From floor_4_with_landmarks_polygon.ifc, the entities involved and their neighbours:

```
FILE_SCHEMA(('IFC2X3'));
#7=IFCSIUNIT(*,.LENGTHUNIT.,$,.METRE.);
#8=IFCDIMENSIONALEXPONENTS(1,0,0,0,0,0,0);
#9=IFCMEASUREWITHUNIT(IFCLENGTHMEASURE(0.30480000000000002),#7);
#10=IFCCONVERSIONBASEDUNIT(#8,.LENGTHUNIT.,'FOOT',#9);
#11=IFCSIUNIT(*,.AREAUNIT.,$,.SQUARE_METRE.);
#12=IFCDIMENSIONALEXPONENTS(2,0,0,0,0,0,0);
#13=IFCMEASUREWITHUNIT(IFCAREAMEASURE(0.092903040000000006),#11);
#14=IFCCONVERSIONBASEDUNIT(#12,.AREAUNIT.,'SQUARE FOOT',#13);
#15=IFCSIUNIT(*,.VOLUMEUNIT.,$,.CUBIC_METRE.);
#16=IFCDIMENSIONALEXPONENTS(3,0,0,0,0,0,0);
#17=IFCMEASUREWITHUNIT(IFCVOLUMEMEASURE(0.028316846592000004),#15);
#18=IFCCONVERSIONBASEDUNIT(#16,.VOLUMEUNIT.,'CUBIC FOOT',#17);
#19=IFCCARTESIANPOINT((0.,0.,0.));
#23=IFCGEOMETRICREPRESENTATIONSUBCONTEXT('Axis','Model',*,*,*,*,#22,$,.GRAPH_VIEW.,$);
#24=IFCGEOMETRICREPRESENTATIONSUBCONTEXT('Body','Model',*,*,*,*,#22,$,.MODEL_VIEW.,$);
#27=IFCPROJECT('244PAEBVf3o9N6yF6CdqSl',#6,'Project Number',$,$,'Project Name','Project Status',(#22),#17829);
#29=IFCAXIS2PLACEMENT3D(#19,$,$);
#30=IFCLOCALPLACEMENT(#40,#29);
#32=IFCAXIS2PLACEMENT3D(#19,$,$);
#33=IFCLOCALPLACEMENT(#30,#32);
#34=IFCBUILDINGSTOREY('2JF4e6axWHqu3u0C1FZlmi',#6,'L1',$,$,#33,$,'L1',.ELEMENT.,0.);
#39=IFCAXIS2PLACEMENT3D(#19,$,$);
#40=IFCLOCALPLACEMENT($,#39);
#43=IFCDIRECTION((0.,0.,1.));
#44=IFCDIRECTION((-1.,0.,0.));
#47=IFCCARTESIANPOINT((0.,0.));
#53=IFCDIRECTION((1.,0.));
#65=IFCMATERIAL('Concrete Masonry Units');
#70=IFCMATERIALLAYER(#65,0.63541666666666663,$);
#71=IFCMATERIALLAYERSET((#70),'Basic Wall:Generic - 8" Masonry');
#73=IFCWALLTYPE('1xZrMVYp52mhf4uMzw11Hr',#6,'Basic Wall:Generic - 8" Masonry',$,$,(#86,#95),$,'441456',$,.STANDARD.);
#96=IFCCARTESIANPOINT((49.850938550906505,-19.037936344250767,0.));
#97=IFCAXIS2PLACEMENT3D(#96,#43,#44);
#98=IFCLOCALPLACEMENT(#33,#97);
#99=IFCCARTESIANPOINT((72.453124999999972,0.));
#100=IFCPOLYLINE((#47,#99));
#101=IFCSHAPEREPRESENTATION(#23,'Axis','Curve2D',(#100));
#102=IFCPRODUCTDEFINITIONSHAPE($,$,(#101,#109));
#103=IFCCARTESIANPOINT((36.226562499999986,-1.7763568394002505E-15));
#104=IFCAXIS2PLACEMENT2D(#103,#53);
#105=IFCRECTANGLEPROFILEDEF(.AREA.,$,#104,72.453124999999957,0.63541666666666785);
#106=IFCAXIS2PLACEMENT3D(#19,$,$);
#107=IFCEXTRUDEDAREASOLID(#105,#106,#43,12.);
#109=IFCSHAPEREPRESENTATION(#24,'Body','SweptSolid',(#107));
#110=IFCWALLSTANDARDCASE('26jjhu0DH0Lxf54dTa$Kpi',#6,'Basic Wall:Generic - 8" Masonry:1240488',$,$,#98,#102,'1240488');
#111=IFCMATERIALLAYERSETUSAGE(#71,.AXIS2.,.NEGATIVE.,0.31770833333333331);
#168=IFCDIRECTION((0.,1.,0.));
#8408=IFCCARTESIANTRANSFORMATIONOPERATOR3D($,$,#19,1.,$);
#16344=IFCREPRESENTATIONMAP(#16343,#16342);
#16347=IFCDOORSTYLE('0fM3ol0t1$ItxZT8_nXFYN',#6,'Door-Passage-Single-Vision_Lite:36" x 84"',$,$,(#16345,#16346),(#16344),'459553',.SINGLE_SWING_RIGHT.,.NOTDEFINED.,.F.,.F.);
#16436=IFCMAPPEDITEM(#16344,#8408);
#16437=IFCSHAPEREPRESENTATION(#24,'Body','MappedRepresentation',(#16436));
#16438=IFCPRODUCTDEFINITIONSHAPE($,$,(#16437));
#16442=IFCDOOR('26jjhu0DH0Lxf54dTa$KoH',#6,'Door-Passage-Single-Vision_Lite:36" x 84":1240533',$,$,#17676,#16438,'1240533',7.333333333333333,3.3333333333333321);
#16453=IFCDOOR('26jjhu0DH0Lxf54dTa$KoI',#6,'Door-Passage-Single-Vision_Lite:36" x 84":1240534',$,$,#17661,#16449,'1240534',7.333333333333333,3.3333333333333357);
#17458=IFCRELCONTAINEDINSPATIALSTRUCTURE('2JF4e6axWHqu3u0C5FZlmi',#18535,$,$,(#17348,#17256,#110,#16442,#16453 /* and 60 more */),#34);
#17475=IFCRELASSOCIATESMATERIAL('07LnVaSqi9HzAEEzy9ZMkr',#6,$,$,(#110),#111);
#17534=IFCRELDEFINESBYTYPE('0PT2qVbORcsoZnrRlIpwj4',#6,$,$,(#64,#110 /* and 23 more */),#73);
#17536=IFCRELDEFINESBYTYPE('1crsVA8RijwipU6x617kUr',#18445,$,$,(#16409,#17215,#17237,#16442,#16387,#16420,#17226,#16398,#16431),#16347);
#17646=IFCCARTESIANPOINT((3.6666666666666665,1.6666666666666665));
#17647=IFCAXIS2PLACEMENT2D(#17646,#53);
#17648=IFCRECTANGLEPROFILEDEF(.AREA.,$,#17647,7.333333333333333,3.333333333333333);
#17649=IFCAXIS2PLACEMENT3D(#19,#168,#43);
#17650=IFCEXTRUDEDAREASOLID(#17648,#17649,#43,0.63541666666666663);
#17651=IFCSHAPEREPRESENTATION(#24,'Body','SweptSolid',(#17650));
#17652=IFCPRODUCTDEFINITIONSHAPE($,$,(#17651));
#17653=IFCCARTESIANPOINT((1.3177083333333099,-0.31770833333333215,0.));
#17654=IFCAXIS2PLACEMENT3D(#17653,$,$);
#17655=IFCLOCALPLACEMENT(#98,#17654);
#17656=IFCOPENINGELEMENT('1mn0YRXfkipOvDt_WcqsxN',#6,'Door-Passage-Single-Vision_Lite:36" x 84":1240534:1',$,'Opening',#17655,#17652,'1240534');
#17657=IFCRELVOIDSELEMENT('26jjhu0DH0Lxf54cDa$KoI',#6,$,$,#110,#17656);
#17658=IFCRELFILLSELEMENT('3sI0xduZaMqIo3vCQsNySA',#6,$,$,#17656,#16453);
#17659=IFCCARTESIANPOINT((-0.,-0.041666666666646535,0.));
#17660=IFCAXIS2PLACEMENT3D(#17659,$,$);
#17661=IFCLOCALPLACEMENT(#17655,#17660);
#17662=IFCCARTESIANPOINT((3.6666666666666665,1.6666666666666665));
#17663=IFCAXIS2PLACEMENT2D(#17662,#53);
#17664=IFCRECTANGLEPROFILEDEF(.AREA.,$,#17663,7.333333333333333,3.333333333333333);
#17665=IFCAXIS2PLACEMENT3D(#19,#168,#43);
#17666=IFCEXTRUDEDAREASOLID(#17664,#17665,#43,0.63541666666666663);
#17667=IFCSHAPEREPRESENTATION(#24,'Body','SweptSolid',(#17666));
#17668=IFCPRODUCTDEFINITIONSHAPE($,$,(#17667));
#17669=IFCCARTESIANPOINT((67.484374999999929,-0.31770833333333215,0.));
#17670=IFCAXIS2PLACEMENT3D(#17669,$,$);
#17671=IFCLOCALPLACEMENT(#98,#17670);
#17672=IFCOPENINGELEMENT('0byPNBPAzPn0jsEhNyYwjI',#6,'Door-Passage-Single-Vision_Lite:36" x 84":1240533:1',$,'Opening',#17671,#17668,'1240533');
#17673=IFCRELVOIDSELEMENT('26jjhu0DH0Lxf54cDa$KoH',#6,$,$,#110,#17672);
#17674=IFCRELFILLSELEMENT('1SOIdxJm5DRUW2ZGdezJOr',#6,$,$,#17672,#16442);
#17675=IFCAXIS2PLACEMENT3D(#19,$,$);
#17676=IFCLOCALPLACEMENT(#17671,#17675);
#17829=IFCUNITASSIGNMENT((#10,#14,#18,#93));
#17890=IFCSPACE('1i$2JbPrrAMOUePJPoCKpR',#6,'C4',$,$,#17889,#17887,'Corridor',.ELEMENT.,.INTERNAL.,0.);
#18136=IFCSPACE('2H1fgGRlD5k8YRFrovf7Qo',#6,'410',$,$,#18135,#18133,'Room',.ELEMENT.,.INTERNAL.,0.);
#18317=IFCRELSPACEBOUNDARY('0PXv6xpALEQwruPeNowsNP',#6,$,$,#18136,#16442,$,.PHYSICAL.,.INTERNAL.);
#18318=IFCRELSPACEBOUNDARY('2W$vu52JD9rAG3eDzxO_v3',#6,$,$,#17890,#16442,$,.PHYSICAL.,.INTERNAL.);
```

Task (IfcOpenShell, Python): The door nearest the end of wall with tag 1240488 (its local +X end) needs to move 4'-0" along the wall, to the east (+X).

```python
import ifcopenshell
import ifcopenshell.api.geometry
import ifcopenshell.util.placement
import ifcopenshell.util.unit

model = ifcopenshell.open("floor_4_with_landmarks_polygon.ifc")
unit_scale = ifcopenshell.util.unit.calculate_unit_scale(model)

door = model.by_id(16442)
opening = door.FillsVoids[0].RelatingOpeningElement
wall = opening.VoidsElements[0].RelatingBuildingElement

wall_matrix = ifcopenshell.util.placement.get_local_placement(wall.ObjectPlacement)
shift = wall_matrix[:3, 0] * -48 * 0.0254 / unit_scale
before = ifcopenshell.util.placement.get_local_placement(door.ObjectPlacement)[:3, 3].copy()

# The door is placed relative to its opening, so it follows when the opening moves.
matrix = ifcopenshell.util.placement.get_local_placement(opening.ObjectPlacement)
matrix[:3, 3] += shift
ifcopenshell.api.geometry.edit_object_placement(
    model, product=opening, matrix=matrix, is_si=False, should_transform_children=True
)

after = ifcopenshell.util.placement.get_local_placement(door.ObjectPlacement)[:3, 3]
print("door moved by", (after - before).round(3) + 0.0)

model.write("floor_4_with_landmarks_polygon_v2.ifc")
```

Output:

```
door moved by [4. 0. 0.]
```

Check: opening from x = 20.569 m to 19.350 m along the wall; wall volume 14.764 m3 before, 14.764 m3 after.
